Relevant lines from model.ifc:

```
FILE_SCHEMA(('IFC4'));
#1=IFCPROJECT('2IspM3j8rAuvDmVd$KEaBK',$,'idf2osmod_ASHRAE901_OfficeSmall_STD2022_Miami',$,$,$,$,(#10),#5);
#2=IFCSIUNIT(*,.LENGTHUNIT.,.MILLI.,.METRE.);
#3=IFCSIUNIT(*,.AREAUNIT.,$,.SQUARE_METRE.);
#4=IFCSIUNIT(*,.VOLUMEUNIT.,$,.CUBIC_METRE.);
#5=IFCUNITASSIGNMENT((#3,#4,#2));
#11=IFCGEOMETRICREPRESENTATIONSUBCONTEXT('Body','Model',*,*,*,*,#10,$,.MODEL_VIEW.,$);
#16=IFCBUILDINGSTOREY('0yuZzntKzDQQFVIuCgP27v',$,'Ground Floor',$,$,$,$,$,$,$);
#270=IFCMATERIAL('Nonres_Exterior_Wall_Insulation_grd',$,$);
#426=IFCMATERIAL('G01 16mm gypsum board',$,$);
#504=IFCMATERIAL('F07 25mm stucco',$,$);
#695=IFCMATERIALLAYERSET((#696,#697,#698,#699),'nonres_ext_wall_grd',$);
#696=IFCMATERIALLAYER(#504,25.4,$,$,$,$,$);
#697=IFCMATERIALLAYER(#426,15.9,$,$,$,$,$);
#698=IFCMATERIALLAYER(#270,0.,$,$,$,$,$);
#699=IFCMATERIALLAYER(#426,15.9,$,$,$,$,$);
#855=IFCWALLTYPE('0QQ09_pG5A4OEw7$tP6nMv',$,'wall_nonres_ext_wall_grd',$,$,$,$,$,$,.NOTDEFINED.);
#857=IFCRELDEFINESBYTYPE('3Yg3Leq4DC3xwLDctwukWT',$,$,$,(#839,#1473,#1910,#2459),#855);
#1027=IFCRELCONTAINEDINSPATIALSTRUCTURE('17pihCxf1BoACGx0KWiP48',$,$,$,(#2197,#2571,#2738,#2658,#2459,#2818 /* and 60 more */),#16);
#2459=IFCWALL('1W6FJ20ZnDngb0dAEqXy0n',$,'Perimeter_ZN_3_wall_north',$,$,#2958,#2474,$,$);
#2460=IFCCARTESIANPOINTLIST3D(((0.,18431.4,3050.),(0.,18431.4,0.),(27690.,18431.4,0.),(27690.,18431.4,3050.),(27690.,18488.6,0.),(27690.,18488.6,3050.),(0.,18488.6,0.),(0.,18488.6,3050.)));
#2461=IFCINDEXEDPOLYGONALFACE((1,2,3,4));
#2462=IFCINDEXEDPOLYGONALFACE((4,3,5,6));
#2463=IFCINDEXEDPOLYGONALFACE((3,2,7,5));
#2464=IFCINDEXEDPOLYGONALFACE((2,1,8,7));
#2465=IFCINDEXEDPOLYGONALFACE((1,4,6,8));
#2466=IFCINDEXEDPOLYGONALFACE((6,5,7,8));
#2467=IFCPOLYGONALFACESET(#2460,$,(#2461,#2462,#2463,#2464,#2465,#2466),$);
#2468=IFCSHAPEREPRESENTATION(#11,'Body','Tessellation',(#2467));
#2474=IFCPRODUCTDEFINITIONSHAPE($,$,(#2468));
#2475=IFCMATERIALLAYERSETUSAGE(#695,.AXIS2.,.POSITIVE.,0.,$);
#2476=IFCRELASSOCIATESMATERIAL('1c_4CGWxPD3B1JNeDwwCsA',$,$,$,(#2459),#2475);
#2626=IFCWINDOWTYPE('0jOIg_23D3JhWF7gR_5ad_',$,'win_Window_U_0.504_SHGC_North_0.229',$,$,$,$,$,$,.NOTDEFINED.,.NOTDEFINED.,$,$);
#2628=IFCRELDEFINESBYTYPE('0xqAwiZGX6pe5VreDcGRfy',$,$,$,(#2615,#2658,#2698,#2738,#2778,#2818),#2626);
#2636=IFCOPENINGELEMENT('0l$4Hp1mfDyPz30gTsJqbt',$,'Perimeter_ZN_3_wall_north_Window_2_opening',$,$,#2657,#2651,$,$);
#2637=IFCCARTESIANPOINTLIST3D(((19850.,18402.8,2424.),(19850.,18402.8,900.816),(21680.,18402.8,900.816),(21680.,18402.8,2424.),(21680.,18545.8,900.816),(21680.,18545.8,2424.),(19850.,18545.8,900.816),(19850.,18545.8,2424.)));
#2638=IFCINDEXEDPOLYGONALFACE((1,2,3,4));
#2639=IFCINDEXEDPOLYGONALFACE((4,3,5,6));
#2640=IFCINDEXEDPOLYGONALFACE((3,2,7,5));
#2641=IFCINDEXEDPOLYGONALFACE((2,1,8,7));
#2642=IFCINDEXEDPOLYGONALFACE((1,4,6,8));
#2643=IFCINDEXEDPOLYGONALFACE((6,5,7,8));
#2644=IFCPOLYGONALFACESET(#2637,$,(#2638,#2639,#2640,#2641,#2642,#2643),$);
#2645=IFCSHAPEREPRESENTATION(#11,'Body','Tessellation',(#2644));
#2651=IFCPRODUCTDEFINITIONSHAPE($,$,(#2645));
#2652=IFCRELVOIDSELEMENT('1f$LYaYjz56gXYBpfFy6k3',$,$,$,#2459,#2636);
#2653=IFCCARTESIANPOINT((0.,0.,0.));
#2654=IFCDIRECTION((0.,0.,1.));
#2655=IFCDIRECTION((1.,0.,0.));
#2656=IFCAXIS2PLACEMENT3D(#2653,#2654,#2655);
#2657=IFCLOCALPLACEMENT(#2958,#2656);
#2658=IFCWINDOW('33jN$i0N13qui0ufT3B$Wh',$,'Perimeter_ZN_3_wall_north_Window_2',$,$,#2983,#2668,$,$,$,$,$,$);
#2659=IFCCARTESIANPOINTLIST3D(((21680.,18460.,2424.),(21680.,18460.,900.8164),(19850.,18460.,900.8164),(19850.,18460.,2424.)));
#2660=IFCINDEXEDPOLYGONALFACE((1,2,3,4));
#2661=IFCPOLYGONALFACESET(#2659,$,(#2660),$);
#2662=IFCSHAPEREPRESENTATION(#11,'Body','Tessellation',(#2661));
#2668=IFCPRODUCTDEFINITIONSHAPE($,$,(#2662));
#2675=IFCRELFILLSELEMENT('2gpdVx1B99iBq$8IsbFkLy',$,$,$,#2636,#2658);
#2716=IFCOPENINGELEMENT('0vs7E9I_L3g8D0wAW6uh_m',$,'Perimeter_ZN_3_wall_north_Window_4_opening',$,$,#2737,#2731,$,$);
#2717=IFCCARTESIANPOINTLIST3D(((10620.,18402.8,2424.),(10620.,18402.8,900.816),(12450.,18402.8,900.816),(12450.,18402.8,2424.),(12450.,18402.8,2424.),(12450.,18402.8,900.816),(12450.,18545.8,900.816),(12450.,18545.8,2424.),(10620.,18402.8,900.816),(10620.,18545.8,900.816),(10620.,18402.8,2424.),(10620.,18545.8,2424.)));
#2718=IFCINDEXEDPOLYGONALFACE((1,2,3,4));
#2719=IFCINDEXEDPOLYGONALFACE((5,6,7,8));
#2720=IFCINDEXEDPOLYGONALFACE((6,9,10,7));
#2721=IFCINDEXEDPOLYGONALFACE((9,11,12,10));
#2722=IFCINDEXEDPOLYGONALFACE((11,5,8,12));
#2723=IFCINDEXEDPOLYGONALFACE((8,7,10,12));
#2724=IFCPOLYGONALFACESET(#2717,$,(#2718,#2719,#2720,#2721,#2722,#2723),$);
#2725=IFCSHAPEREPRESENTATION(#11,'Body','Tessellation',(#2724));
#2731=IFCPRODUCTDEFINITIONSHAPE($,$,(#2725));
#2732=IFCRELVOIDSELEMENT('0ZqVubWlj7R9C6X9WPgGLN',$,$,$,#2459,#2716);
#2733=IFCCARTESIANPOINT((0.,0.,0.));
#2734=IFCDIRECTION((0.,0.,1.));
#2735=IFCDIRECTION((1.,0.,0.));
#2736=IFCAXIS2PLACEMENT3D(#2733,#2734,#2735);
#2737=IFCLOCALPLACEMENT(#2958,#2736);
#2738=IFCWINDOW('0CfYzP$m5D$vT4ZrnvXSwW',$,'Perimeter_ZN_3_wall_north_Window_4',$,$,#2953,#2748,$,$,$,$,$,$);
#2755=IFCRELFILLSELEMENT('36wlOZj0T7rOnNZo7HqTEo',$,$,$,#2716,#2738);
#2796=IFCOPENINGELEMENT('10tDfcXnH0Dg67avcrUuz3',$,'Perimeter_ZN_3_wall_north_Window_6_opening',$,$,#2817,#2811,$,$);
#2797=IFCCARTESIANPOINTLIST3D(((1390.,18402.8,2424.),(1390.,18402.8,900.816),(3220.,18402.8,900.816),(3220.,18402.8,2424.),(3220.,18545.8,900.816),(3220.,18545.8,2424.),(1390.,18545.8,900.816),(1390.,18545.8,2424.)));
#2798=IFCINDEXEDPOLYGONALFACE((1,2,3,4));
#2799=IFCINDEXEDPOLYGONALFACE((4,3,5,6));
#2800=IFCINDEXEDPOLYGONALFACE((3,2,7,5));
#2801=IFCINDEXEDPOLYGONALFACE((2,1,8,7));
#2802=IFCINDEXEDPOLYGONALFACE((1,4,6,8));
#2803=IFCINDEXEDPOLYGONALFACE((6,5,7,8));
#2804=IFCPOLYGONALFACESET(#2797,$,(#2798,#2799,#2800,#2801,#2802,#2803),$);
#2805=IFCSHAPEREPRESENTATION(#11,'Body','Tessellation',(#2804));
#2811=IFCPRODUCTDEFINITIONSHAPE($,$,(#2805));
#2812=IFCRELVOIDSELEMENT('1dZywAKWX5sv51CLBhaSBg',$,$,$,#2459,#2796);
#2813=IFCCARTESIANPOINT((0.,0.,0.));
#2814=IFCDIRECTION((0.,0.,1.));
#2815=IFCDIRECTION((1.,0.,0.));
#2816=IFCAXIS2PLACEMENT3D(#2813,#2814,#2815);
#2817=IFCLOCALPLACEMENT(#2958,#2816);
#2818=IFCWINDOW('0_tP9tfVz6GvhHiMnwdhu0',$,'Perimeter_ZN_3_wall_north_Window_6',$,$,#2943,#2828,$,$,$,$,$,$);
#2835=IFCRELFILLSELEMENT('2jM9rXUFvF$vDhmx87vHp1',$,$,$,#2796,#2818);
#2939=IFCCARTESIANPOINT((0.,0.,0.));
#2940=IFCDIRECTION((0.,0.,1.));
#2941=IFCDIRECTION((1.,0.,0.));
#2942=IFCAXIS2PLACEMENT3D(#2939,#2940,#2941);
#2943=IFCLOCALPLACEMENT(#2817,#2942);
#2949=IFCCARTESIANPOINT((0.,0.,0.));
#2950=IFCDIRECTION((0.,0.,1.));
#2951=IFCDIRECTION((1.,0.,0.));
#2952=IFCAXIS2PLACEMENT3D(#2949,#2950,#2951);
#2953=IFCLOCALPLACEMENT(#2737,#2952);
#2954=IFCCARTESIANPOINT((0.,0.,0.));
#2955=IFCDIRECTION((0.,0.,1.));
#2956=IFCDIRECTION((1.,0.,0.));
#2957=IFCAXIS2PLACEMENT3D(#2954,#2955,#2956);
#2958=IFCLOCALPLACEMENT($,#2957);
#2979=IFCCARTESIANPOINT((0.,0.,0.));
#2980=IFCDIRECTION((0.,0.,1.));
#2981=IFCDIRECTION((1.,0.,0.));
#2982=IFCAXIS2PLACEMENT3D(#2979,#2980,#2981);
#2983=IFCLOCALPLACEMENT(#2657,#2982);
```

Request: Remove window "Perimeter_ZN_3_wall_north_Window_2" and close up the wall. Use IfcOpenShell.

```python
import ifcopenshell
import ifcopenshell.api.feature
import ifcopenshell.api.root
import ifcopenshell.geom
import ifcopenshell.util.shape

model = ifcopenshell.open("model.ifc")
settings = ifcopenshell.geom.settings()


def volume(element):
    """Net volume in cubic metres, openings subtracted."""
    shape = ifcopenshell.geom.create_shape(settings, element)
    return ifcopenshell.util.shape.get_volume(shape.geometry)


window = model.by_guid("33jN$i0N13qui0ufT3B$Wh")
opening = window.FillsVoids[0].RelatingOpeningElement
wall = opening.VoidsElements[0].RelatingBuildingElement
before = volume(wall)

ifcopenshell.api.root.remove_product(model, product=window)
ifcopenshell.api.feature.remove_feature(model, feature=opening)

after = volume(wall)

print(f"wall volume {before:.3f} -> {after:.3f} m3")

model.write("model-out.ifc")
```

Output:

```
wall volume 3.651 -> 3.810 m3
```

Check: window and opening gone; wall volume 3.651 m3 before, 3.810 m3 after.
